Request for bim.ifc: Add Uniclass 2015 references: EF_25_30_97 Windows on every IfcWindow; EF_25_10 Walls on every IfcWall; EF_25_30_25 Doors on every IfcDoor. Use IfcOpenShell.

First a look at what the model holds.

```python
import ifcopenshell

model = ifcopenshell.open("bim.ifc")
print(model.schema)
print("classifications:", [c.Name for c in model.by_type("IfcClassification")])
for ifc_class in ("IfcDoor", "IfcRoof", "IfcStair", "IfcWall", "IfcWindow"):
    print(ifc_class, len(model.by_type(ifc_class)))
```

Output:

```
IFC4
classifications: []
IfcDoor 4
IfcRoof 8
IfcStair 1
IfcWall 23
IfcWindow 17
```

```python
import ifcopenshell
import ifcopenshell.api.classification

model = ifcopenshell.open("bim.ifc")

system = ifcopenshell.api.classification.add_classification(model, classification="Uniclass 2015")

codes = {
    "IfcWindow": ("EF_25_30_97", "Windows"),
    "IfcWall": ("EF_25_10", "Walls"),
    "IfcDoor": ("EF_25_30_25", "Doors"),
}
for ifc_class, (code, name) in codes.items():
    products = model.by_type(ifc_class)
    ifcopenshell.api.classification.add_reference(
        model, products=products, classification=system, identification=code, name=name
    )
    print(code, len(products))

model.write("bim_updated.ifc")
```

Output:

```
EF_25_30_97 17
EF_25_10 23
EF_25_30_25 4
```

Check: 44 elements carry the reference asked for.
